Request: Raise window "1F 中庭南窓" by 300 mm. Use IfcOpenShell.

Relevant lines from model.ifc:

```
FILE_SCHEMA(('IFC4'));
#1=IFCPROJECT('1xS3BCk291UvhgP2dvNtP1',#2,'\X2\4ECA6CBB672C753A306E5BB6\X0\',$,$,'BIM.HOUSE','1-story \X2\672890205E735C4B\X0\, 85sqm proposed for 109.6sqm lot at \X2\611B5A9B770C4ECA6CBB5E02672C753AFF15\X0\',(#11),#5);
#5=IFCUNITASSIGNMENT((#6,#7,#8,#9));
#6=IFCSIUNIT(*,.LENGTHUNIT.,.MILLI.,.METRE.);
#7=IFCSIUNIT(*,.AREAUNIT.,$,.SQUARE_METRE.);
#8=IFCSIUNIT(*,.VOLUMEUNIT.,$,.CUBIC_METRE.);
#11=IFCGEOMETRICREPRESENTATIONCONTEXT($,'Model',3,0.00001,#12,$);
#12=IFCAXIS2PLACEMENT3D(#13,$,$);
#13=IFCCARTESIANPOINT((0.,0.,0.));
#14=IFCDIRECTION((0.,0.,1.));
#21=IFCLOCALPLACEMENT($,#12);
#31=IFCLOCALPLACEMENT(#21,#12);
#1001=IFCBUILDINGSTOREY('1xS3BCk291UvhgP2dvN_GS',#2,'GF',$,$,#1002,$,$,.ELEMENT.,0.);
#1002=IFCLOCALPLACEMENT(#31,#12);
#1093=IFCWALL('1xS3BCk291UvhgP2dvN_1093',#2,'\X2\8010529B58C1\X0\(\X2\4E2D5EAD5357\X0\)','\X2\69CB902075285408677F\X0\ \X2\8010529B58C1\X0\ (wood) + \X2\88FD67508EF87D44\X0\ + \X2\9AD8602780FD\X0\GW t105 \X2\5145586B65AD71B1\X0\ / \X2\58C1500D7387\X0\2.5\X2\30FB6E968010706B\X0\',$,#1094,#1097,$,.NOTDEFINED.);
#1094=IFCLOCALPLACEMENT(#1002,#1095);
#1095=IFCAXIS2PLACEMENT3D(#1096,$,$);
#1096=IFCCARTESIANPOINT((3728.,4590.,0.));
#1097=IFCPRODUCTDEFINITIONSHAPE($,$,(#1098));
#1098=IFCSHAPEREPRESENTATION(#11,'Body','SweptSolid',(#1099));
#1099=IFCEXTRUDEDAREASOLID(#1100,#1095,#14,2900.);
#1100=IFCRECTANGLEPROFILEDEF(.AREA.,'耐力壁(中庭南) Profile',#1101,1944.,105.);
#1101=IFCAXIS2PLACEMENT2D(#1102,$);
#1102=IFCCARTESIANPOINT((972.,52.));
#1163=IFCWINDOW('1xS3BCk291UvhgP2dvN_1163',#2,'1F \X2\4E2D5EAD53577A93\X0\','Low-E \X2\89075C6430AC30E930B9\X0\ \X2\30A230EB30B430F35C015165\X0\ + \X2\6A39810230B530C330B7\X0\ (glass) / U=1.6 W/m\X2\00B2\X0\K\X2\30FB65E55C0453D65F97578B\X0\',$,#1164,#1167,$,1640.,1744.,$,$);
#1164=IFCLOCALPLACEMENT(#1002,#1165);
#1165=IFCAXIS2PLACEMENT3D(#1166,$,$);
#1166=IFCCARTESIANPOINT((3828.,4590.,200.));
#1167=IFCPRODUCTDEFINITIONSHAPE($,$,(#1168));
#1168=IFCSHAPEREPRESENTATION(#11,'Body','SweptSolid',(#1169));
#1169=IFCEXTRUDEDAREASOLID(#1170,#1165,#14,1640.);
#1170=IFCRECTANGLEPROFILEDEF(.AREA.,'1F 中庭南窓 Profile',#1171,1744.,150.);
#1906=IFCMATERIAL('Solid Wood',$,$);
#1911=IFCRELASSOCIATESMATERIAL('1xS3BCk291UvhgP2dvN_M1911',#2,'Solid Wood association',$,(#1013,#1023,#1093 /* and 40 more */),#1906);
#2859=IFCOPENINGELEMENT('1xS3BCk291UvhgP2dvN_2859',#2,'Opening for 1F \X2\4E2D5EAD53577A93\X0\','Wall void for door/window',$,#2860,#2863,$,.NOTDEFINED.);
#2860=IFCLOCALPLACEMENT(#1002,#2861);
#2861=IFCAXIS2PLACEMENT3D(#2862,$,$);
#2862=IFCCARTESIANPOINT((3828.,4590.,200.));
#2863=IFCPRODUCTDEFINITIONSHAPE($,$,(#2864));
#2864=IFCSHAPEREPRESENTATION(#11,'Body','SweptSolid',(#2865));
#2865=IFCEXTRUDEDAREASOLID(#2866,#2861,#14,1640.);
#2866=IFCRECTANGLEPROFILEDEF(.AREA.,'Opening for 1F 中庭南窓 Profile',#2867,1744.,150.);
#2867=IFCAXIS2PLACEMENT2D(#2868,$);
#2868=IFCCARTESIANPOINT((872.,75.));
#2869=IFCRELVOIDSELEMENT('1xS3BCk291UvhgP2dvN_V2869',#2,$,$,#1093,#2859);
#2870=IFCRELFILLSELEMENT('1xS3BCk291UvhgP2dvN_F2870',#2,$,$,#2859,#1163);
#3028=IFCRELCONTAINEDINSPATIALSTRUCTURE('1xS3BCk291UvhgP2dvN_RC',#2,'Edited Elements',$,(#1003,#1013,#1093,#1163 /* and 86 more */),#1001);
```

```python
import numpy as np
import ifcopenshell
import ifcopenshell.api.geometry
import ifcopenshell.util.placement
import ifcopenshell.util.unit

model = ifcopenshell.open("model.ifc")
unit_scale = ifcopenshell.util.unit.calculate_unit_scale(model)

window = model.by_id(1163)
opening = window.FillsVoids[0].RelatingOpeningElement
dz = 0.3 / unit_scale

shift = np.array([0.0, 0.0, dz])
# The window is not placed relative to its opening, so move both.
for product in (opening, window):
    matrix = ifcopenshell.util.placement.get_local_placement(product.ObjectPlacement)
    matrix[:3, 3] += shift
    ifcopenshell.api.geometry.edit_object_placement(model, product=product, matrix=matrix, is_si=False)

print(f"moved by {dz * unit_scale:+.3f} m")

model.write("model_updated.ifc")
```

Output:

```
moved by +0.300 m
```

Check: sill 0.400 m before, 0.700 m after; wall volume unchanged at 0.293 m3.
